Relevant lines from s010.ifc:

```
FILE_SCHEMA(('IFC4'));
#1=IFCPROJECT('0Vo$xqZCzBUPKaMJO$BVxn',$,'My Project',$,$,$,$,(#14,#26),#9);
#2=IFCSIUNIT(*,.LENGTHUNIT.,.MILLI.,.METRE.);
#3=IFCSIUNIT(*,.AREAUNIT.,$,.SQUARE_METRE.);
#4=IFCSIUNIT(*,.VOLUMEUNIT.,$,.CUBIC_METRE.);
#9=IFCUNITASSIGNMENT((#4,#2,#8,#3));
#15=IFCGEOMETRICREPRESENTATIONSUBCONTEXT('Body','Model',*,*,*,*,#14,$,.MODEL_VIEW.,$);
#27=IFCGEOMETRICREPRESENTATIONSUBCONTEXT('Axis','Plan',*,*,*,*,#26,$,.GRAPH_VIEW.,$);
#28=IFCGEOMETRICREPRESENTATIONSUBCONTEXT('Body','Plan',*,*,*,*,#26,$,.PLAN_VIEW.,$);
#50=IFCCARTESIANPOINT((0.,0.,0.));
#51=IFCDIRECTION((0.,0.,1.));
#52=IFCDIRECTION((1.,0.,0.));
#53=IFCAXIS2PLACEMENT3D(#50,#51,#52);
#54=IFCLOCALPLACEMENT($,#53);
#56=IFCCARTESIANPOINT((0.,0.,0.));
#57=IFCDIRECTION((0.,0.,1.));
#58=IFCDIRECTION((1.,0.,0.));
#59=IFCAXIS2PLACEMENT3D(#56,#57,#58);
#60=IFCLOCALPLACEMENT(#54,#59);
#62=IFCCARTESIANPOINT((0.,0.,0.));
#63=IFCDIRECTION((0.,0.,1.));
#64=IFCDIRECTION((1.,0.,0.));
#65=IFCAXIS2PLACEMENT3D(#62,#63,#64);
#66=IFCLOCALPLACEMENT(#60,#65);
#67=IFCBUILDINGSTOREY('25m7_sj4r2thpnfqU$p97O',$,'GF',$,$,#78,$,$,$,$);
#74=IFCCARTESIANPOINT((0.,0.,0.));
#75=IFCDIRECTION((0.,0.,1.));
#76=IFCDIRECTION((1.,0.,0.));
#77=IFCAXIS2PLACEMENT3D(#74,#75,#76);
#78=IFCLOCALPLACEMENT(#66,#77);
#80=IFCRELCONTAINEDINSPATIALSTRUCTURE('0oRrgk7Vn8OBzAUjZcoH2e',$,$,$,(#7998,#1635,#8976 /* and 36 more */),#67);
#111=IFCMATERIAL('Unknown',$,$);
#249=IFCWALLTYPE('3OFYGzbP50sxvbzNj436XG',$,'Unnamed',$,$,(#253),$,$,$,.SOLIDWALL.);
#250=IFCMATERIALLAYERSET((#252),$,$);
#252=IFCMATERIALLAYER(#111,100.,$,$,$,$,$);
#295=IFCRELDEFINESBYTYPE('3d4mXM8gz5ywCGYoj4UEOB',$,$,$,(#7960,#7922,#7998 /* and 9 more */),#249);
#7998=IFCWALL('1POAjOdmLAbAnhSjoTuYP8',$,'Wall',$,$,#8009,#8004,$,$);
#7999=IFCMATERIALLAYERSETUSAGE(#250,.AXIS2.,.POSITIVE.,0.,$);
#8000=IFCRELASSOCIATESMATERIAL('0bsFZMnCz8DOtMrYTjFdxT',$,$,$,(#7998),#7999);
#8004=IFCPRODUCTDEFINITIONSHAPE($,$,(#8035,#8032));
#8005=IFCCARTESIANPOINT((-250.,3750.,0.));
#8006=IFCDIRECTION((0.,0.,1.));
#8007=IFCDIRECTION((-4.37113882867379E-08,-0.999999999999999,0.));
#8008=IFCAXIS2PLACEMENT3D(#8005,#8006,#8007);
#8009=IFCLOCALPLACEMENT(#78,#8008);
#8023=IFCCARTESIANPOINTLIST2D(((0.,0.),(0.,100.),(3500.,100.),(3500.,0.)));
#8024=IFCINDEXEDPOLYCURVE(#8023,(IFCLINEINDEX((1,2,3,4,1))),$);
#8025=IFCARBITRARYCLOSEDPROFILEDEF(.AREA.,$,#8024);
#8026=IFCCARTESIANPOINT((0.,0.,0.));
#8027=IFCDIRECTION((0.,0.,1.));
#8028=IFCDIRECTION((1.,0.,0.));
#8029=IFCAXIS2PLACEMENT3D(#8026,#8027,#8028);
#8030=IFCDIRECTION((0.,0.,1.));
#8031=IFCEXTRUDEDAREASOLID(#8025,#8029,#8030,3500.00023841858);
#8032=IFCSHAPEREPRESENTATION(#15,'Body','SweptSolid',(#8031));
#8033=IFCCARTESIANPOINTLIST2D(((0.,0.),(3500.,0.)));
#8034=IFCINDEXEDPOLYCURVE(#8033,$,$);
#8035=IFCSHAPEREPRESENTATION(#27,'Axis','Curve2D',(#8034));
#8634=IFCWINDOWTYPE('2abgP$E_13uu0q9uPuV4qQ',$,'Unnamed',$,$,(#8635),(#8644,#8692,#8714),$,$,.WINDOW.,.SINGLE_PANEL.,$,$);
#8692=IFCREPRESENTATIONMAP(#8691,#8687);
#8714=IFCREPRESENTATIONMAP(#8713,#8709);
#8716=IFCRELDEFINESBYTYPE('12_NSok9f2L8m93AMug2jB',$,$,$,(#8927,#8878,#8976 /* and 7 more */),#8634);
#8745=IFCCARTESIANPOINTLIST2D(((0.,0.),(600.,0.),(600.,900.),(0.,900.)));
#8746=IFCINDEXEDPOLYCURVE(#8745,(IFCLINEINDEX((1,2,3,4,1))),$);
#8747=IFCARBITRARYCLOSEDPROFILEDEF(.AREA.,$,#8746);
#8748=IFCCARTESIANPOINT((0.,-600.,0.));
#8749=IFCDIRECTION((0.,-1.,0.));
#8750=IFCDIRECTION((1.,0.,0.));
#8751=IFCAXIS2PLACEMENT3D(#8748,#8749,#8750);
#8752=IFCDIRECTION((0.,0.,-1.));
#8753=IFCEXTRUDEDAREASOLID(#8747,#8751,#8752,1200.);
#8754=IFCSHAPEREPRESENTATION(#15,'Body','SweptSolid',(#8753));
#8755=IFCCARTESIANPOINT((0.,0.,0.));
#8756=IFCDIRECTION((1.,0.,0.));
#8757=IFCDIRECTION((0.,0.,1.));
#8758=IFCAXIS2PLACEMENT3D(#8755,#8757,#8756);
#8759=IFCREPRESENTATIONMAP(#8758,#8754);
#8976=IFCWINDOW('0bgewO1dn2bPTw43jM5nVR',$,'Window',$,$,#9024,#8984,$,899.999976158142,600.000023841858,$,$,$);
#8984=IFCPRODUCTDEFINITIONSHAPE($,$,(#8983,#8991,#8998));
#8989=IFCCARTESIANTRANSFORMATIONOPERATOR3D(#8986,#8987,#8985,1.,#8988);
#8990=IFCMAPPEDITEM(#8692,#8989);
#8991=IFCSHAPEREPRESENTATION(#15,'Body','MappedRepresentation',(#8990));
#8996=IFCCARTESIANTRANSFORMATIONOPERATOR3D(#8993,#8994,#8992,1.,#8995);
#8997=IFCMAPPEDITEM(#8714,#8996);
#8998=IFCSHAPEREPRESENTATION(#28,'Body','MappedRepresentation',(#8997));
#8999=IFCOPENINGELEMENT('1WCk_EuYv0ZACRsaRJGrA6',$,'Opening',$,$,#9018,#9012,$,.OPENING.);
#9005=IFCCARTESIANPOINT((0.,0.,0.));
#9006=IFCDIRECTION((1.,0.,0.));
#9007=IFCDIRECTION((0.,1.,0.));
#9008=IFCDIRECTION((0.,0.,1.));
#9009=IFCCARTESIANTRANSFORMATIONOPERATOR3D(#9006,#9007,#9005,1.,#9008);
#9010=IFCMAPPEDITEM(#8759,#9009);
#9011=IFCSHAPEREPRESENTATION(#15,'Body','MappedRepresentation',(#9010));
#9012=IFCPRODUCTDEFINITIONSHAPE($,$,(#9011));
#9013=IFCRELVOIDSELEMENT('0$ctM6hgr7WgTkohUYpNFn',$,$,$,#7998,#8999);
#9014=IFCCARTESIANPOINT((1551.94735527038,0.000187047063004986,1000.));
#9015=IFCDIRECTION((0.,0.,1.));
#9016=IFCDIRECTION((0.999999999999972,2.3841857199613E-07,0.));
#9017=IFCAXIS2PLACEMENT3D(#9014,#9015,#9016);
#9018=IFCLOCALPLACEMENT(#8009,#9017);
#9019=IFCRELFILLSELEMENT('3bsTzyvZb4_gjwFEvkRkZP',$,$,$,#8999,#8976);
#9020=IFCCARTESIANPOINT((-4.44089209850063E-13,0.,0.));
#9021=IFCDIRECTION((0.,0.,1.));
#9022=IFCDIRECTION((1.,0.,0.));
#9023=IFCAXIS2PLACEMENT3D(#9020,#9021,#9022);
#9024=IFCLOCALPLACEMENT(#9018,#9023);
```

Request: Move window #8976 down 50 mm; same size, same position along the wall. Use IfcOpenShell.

```python
import numpy as np
import ifcopenshell
import ifcopenshell.api.geometry
import ifcopenshell.util.placement
import ifcopenshell.util.unit

model = ifcopenshell.open("s010.ifc")
unit_scale = ifcopenshell.util.unit.calculate_unit_scale(model)

window = model.by_guid("0bgewO1dn2bPTw43jM5nVR")
opening = window.FillsVoids[0].RelatingOpeningElement
dz = -0.05 / unit_scale

shift = np.array([0.0, 0.0, dz])
# The window is placed relative to its opening, so it follows when the opening moves.
matrix = ifcopenshell.util.placement.get_local_placement(opening.ObjectPlacement)
matrix[:3, 3] += shift
ifcopenshell.api.geometry.edit_object_placement(
    model, product=opening, matrix=matrix, is_si=False, should_transform_children=True
)

print(f"moved by {dz * unit_scale:+.3f} m")

model.write("s010_rev.ifc")
```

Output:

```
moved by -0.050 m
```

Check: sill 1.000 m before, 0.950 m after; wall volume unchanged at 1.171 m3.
